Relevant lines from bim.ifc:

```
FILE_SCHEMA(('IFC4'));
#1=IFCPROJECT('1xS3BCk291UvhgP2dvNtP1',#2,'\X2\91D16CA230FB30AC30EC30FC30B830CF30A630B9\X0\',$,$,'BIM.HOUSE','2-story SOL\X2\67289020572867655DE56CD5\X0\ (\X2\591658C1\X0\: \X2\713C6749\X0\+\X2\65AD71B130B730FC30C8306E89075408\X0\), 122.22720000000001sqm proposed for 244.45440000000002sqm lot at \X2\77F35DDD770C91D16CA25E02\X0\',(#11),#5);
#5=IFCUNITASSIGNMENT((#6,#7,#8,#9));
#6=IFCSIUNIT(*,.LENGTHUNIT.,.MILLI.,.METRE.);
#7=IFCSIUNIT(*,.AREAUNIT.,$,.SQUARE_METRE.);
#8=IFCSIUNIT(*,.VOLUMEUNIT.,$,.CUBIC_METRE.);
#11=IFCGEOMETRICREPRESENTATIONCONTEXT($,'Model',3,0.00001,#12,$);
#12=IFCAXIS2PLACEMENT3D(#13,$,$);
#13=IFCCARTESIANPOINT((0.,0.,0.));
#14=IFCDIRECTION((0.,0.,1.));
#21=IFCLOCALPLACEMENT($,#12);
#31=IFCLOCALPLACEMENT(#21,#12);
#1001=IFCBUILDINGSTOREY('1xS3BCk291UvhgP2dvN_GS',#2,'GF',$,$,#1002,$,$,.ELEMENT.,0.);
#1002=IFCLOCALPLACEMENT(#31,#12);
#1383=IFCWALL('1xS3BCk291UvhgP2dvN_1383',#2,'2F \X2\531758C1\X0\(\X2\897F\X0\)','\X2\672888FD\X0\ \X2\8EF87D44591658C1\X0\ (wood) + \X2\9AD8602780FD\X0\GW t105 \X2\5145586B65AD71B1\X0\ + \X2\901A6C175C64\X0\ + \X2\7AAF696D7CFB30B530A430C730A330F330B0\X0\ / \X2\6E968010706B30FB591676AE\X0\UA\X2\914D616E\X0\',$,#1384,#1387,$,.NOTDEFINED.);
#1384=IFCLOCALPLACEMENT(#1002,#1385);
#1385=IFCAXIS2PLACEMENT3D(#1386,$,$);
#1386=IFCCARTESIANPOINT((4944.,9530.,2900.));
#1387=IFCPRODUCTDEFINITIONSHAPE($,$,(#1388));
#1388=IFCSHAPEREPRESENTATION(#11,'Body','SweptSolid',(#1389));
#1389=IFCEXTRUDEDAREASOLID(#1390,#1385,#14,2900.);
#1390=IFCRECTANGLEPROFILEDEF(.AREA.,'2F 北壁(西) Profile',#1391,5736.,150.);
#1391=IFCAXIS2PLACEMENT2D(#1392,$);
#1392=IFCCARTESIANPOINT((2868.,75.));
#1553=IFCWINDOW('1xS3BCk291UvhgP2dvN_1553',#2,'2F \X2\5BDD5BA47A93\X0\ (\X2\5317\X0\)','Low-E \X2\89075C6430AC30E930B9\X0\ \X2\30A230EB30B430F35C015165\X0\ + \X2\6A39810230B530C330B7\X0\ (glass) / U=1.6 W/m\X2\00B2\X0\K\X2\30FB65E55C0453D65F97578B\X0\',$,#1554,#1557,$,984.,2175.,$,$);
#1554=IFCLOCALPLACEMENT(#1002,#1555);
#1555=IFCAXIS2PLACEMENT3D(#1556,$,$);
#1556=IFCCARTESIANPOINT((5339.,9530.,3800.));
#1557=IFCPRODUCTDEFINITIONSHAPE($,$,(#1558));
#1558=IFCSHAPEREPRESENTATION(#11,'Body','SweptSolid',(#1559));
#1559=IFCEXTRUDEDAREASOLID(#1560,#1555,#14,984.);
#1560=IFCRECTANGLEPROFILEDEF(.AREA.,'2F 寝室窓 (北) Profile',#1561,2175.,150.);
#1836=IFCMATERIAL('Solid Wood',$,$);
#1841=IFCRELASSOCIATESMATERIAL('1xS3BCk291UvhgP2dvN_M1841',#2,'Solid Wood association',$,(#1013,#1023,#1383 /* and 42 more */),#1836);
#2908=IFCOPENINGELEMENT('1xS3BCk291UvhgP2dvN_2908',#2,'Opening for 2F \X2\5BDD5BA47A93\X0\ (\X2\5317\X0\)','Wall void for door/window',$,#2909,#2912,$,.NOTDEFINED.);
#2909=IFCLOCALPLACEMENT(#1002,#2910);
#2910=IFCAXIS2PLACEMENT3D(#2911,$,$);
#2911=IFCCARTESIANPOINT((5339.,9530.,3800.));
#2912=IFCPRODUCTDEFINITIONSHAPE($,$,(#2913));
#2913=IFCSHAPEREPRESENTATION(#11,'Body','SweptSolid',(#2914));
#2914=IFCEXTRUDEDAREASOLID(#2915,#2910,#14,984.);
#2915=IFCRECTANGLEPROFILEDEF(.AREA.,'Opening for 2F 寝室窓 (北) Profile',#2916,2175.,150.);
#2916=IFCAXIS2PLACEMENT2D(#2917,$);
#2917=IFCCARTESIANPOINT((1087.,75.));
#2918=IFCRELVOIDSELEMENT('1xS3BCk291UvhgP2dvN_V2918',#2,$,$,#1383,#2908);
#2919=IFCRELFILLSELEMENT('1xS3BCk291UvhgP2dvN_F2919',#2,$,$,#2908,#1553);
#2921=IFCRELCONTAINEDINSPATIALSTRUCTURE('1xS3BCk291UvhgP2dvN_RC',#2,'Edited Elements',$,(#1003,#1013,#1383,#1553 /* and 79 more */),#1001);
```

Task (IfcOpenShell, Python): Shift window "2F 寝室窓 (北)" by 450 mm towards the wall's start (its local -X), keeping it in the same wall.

```python
import ifcopenshell
import ifcopenshell.api.geometry
import ifcopenshell.util.placement

model = ifcopenshell.open("bim.ifc")

window = model.by_id(1553)
opening = window.FillsVoids[0].RelatingOpeningElement
wall = opening.VoidsElements[0].RelatingBuildingElement

wall_matrix = ifcopenshell.util.placement.get_local_placement(wall.ObjectPlacement)
shift = wall_matrix[:3, 0] * -450.0
before = ifcopenshell.util.placement.get_local_placement(window.ObjectPlacement)[:3, 3].copy()

# The window is not placed relative to its opening, so move both.
for product in (opening, window):
    matrix = ifcopenshell.util.placement.get_local_placement(product.ObjectPlacement)
    matrix[:3, 3] += shift
    ifcopenshell.api.geometry.edit_object_placement(model, product=product, matrix=matrix, is_si=False)

after = ifcopenshell.util.placement.get_local_placement(window.ObjectPlacement)[:3, 3]
print("window moved by", (after - before).round(3) + 0.0)

model.write("bim-out.ifc")
```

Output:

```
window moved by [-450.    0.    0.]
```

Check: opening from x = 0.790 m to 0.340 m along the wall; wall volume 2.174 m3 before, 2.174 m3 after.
